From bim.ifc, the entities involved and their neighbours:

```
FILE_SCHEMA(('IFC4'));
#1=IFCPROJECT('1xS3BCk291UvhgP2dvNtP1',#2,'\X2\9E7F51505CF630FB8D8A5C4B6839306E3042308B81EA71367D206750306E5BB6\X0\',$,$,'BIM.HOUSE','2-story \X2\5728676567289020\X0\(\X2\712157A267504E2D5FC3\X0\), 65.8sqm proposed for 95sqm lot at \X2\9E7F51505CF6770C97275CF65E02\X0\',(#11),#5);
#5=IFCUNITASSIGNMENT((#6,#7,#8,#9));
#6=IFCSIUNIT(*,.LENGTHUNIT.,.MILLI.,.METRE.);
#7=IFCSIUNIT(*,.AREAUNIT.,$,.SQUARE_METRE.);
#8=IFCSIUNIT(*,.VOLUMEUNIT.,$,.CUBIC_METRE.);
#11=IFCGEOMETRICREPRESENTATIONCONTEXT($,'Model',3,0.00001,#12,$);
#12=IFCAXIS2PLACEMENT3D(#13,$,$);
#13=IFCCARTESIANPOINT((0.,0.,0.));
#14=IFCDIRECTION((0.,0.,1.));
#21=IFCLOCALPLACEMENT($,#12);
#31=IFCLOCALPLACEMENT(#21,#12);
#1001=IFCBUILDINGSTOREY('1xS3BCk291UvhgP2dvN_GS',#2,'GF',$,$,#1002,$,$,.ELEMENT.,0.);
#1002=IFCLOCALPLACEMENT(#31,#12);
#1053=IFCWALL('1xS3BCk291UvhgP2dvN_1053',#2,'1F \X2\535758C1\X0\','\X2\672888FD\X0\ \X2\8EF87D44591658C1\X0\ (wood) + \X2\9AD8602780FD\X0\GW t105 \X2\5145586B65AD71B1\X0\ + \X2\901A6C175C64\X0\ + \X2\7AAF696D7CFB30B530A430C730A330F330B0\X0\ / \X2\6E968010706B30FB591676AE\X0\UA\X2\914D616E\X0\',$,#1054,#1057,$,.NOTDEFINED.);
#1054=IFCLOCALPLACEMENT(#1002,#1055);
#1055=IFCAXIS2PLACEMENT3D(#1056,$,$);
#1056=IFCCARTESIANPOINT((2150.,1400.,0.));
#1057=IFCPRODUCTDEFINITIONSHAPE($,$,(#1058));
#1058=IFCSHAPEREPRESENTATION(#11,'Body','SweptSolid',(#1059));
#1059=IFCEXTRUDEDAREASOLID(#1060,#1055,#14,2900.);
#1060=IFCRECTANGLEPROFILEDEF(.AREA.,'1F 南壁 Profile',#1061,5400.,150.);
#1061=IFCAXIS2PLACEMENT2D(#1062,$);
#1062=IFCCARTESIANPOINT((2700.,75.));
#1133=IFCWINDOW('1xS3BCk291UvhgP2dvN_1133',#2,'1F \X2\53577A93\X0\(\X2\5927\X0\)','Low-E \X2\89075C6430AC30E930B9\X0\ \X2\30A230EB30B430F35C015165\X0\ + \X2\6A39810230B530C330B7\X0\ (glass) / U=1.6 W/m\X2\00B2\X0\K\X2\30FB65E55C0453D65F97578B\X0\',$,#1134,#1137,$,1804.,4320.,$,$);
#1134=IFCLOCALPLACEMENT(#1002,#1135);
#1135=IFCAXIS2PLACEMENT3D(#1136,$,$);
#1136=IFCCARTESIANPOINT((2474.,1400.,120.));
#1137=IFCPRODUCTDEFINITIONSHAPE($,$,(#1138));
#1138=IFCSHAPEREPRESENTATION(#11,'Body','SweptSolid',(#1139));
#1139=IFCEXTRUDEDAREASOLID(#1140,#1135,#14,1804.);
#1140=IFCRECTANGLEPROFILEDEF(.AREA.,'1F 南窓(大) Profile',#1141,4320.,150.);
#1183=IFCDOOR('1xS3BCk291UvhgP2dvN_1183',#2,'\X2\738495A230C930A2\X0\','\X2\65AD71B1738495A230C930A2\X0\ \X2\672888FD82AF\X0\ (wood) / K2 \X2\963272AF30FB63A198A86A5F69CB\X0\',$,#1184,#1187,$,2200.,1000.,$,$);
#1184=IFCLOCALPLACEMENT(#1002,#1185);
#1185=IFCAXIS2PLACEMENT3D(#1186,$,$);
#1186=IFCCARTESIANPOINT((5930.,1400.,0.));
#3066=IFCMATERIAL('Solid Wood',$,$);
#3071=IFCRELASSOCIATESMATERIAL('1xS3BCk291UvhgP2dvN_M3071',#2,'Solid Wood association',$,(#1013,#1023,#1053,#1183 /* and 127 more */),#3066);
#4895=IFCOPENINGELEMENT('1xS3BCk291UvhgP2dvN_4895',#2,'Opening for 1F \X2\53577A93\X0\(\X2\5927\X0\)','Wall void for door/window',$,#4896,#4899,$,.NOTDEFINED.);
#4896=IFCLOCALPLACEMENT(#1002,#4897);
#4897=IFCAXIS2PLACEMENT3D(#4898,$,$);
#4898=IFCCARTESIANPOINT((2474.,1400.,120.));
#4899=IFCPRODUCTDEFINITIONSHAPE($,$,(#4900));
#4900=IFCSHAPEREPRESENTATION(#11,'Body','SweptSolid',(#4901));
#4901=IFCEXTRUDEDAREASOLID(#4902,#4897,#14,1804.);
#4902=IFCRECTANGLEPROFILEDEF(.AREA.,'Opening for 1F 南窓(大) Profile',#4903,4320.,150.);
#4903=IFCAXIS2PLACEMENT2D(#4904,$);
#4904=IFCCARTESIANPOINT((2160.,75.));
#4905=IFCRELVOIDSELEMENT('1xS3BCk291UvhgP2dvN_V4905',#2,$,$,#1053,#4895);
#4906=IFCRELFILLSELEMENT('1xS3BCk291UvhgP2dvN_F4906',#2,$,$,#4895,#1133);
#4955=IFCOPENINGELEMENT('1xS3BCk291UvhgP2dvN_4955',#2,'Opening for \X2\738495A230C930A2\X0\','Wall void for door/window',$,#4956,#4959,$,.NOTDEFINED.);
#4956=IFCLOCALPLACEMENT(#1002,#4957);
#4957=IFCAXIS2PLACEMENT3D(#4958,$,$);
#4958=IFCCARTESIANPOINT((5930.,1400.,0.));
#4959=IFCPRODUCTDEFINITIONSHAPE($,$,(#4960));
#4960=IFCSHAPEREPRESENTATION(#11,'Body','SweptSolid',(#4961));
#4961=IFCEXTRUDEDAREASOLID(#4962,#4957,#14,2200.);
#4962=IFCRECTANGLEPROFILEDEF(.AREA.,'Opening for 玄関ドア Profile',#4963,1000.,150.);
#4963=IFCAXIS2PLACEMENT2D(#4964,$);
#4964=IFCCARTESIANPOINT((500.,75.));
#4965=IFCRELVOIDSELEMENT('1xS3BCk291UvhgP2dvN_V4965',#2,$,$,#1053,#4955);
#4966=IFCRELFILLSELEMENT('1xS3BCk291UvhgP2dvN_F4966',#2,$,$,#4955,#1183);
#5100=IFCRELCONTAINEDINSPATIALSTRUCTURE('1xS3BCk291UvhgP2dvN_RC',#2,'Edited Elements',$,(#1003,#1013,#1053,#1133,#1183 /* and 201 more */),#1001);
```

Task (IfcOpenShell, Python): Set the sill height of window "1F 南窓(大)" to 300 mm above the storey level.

```python
import numpy as np
import ifcopenshell
import ifcopenshell.api.geometry
import ifcopenshell.geom
import ifcopenshell.util.element
import ifcopenshell.util.placement
import ifcopenshell.util.shape
import ifcopenshell.util.unit

model = ifcopenshell.open("bim.ifc")
unit_scale = ifcopenshell.util.unit.calculate_unit_scale(model)

window = model.by_guid("1xS3BCk291UvhgP2dvN_1133")
opening = window.FillsVoids[0].RelatingOpeningElement
storey = ifcopenshell.util.element.get_container(window, ifc_class="IfcBuildingStorey")
level = ifcopenshell.util.placement.get_local_placement(storey.ObjectPlacement)[2, 3]

# The opening's origin need not be at the sill, so measure its lowest point.
shape = ifcopenshell.geom.create_shape(ifcopenshell.geom.settings(), opening)
bottom = ifcopenshell.util.shape.get_shape_bottom_elevation(shape, shape.geometry) / unit_scale
dz = level + 300.0 - bottom

shift = np.array([0.0, 0.0, dz])
# The window is not placed relative to its opening, so move both.
for product in (opening, window):
    matrix = ifcopenshell.util.placement.get_local_placement(product.ObjectPlacement)
    matrix[:3, 3] += shift
    ifcopenshell.api.geometry.edit_object_placement(model, product=product, matrix=matrix, is_si=False)

print(f"moved by {dz * unit_scale:+.3f} m")

model.write("bim_edited.ifc")
```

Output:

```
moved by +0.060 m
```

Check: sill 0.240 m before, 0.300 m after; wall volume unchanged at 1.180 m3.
